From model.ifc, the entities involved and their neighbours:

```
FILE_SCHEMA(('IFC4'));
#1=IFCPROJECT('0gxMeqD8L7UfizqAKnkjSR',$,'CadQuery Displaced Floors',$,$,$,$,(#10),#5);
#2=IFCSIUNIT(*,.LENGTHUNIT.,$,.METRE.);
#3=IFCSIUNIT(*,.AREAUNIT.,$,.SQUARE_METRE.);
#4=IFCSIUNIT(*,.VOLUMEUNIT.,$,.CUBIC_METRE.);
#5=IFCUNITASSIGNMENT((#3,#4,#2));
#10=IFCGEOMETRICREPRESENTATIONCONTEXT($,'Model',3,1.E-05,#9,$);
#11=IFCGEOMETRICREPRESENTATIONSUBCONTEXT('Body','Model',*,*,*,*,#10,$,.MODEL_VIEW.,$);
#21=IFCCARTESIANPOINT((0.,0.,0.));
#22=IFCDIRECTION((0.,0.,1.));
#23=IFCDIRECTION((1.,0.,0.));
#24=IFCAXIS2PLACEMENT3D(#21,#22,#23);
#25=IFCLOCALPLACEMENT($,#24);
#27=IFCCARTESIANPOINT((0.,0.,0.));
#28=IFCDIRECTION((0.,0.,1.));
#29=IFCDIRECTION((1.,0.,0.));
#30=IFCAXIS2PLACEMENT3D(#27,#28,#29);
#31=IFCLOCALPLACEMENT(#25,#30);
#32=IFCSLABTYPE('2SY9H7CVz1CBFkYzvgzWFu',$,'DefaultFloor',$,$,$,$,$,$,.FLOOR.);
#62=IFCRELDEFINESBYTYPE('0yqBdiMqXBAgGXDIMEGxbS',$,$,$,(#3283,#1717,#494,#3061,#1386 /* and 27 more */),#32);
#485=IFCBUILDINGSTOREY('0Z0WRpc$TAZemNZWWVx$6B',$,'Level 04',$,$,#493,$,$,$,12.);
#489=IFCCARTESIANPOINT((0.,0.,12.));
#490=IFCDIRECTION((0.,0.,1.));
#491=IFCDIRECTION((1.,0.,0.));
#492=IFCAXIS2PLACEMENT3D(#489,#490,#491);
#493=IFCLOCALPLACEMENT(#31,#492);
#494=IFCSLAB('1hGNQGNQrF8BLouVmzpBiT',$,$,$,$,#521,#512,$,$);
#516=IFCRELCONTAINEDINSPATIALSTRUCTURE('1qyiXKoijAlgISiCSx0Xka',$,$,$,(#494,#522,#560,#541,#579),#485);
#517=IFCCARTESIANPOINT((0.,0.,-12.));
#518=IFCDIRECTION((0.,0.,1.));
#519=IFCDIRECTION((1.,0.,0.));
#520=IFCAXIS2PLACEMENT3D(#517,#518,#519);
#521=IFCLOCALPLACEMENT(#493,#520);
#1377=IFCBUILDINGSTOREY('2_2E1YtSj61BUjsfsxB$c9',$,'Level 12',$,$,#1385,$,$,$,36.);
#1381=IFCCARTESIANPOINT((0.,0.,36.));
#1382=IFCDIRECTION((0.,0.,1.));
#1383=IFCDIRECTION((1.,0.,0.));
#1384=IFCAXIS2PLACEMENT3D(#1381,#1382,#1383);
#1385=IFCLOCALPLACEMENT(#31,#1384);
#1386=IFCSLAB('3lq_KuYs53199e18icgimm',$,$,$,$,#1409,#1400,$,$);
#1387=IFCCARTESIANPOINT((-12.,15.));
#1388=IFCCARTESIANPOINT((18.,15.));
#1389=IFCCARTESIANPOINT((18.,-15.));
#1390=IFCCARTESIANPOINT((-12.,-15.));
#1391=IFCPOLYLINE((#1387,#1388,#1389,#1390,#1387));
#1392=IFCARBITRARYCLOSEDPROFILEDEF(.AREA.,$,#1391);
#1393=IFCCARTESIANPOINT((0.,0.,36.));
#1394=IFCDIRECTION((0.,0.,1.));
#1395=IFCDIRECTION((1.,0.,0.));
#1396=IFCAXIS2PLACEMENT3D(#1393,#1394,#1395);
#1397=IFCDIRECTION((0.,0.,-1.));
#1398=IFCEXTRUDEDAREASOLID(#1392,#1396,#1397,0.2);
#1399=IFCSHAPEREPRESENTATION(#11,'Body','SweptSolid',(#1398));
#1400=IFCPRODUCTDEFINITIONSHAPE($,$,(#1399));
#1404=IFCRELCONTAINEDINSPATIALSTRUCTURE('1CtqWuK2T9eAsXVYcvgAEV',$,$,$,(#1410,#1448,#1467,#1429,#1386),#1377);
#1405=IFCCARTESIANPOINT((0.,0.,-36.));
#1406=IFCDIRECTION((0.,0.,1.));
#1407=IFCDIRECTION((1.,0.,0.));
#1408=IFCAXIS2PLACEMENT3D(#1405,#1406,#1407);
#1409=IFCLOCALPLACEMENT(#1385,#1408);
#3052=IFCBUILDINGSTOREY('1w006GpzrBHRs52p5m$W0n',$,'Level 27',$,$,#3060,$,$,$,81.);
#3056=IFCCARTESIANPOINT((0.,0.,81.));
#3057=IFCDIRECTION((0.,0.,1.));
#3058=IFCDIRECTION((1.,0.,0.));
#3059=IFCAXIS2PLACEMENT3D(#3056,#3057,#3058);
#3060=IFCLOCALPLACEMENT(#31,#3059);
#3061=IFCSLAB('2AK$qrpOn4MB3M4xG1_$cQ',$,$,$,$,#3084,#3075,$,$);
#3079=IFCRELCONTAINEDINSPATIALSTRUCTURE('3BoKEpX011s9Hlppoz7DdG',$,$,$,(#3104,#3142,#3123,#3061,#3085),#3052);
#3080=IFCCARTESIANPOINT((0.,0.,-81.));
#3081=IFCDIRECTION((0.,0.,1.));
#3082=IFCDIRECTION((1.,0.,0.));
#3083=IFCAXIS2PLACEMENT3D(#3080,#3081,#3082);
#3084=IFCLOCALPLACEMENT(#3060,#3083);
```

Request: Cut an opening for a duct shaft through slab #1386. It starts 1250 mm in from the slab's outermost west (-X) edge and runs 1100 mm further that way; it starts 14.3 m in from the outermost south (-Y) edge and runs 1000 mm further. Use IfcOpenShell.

```python
import numpy as np
import ifcopenshell
import ifcopenshell.api.feature
import ifcopenshell.api.geometry
import ifcopenshell.api.root
import ifcopenshell.geom
import ifcopenshell.util.placement
import ifcopenshell.util.representation
import ifcopenshell.util.shape
import ifcopenshell.util.unit

model = ifcopenshell.open("model.ifc")
unit_scale = ifcopenshell.util.unit.calculate_unit_scale(model)
settings = ifcopenshell.geom.settings()


def volume(element):
    """Net volume in cubic metres, openings subtracted."""
    shape = ifcopenshell.geom.create_shape(settings, element)
    return ifcopenshell.util.shape.get_volume(shape.geometry)


slab = model.by_guid("3lq_KuYs53199e18icgimm")
before = volume(slab)

# Extent in the slab's own axes, in metres. The edges named are its -X and -Y sides.
slab_shape = ifcopenshell.geom.create_shape(settings, slab)
vertices = ifcopenshell.util.shape.get_vertices(slab_shape.geometry)
x_min, y_min, bottom = vertices.min(axis=0)
top = vertices[:, 2].max()

opening = ifcopenshell.api.root.create_entity(model, ifc_class="IfcOpeningElement", name="Duct shaft opening", predefined_type="OPENING")
context = ifcopenshell.util.representation.get_context(model, "Model", "Body", "MODEL_VIEW")
width, depth = 1.1, 1
outline = [(0.0, 0.0), (width, 0.0), (width, depth), (0.0, depth), (0.0, 0.0)]
# Overshoot both faces by 50 mm so the cut is clean.
shape = ifcopenshell.api.geometry.add_slab_representation(
    model, context=context, depth=top - bottom + 0.1, polyline=outline
)
ifcopenshell.api.geometry.assign_representation(model, product=opening, representation=shape)

matrix = ifcopenshell.util.placement.get_local_placement(slab.ObjectPlacement)
matrix[:, 3] = matrix @ np.append(np.array([x_min + 1.25, y_min + 14.3, bottom - 0.05]) / unit_scale, 1.0)
ifcopenshell.api.geometry.edit_object_placement(model, product=opening, matrix=matrix, is_si=False)
ifcopenshell.api.feature.add_feature(model, feature=opening, element=slab)

after = volume(slab)

print(f"slab volume {before:.3f} -> {after:.3f} m3")

model.write("model_v2.ifc")
```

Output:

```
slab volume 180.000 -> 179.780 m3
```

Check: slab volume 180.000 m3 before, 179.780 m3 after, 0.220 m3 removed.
